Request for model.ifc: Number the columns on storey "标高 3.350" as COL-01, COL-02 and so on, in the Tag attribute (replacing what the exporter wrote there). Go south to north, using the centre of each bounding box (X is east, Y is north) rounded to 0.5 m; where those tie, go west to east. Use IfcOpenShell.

First a look at what the model holds.

```python
import ifcopenshell
import ifcopenshell.util.element
import ifcopenshell.util.placement

model = ifcopenshell.open("model.ifc")
print(model.schema)
storey = next(s for s in model.by_type("IfcBuildingStorey") if s.Name == "标高 3.350")
columns = [e for e in ifcopenshell.util.element.get_decomposition(storey) if e.is_a("IfcColumn")]
for e in sorted(columns, key=lambda e: e.id()):
    origin = ifcopenshell.util.placement.get_local_placement(e.ObjectPlacement)[:3, 3]
    print(e.id(), e.Tag, e.Name, origin.round(2) + 0.0, sep=" | ")
```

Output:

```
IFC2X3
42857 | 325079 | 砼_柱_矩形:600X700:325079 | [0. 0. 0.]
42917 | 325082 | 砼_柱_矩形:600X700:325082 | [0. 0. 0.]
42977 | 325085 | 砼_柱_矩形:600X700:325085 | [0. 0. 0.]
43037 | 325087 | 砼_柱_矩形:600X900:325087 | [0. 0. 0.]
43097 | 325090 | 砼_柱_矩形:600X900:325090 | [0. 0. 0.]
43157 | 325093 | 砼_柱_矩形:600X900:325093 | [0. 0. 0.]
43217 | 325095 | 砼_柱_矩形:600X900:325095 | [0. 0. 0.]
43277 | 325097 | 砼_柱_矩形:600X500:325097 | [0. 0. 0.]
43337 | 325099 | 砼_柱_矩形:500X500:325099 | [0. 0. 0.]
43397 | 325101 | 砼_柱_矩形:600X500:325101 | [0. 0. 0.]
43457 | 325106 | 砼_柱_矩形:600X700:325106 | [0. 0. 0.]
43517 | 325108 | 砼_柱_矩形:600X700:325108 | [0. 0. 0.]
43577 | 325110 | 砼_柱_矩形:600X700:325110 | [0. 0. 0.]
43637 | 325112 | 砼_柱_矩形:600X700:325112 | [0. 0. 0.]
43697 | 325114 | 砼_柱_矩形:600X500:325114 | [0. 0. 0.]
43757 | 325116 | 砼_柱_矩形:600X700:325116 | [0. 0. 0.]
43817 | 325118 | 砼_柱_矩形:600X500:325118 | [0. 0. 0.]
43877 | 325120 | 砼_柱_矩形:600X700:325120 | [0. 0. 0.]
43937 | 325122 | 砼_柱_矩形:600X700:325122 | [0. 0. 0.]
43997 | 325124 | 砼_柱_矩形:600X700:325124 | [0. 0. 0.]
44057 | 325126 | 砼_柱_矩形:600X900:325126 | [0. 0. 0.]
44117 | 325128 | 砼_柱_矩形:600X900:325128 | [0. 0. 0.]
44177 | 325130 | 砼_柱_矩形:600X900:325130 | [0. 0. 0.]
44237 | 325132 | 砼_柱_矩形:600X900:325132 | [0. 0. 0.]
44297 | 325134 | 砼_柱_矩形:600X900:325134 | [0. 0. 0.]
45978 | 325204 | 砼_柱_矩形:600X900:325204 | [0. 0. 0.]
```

```python
import ifcopenshell
import ifcopenshell.geom
import ifcopenshell.util.element
import ifcopenshell.util.shape

model = ifcopenshell.open("model.ifc")
settings = ifcopenshell.geom.settings()
settings.set("use-world-coords", True)


def centre(element):
    shape = ifcopenshell.geom.create_shape(settings, element)
    return ifcopenshell.util.shape.get_bbox_centroid(shape.geometry)


storey = next(s for s in model.by_type("IfcBuildingStorey") if s.Name == "标高 3.350")
columns = [e for e in ifcopenshell.util.element.get_decomposition(storey) if e.is_a("IfcColumn")]

# Insertion points can sit at a corner or the storey origin, so sort by the geometry (in metres).
centres = {e: centre(e) for e in columns}
columns.sort(key=lambda e: (round(centres[e][1] / 0.5), centres[e][0]))

for i, e in enumerate(columns, start=1):
    number = f"COL-{i:02d}"
    e.Tag = number
    print(e.id(), number)

model.write("model_edited.ifc")
```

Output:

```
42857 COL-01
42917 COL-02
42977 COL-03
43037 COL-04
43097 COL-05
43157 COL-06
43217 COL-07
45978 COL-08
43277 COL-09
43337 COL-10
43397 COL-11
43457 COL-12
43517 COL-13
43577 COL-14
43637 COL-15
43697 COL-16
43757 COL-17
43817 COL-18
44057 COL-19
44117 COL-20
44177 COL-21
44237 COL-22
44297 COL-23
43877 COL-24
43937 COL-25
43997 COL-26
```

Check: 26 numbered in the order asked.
